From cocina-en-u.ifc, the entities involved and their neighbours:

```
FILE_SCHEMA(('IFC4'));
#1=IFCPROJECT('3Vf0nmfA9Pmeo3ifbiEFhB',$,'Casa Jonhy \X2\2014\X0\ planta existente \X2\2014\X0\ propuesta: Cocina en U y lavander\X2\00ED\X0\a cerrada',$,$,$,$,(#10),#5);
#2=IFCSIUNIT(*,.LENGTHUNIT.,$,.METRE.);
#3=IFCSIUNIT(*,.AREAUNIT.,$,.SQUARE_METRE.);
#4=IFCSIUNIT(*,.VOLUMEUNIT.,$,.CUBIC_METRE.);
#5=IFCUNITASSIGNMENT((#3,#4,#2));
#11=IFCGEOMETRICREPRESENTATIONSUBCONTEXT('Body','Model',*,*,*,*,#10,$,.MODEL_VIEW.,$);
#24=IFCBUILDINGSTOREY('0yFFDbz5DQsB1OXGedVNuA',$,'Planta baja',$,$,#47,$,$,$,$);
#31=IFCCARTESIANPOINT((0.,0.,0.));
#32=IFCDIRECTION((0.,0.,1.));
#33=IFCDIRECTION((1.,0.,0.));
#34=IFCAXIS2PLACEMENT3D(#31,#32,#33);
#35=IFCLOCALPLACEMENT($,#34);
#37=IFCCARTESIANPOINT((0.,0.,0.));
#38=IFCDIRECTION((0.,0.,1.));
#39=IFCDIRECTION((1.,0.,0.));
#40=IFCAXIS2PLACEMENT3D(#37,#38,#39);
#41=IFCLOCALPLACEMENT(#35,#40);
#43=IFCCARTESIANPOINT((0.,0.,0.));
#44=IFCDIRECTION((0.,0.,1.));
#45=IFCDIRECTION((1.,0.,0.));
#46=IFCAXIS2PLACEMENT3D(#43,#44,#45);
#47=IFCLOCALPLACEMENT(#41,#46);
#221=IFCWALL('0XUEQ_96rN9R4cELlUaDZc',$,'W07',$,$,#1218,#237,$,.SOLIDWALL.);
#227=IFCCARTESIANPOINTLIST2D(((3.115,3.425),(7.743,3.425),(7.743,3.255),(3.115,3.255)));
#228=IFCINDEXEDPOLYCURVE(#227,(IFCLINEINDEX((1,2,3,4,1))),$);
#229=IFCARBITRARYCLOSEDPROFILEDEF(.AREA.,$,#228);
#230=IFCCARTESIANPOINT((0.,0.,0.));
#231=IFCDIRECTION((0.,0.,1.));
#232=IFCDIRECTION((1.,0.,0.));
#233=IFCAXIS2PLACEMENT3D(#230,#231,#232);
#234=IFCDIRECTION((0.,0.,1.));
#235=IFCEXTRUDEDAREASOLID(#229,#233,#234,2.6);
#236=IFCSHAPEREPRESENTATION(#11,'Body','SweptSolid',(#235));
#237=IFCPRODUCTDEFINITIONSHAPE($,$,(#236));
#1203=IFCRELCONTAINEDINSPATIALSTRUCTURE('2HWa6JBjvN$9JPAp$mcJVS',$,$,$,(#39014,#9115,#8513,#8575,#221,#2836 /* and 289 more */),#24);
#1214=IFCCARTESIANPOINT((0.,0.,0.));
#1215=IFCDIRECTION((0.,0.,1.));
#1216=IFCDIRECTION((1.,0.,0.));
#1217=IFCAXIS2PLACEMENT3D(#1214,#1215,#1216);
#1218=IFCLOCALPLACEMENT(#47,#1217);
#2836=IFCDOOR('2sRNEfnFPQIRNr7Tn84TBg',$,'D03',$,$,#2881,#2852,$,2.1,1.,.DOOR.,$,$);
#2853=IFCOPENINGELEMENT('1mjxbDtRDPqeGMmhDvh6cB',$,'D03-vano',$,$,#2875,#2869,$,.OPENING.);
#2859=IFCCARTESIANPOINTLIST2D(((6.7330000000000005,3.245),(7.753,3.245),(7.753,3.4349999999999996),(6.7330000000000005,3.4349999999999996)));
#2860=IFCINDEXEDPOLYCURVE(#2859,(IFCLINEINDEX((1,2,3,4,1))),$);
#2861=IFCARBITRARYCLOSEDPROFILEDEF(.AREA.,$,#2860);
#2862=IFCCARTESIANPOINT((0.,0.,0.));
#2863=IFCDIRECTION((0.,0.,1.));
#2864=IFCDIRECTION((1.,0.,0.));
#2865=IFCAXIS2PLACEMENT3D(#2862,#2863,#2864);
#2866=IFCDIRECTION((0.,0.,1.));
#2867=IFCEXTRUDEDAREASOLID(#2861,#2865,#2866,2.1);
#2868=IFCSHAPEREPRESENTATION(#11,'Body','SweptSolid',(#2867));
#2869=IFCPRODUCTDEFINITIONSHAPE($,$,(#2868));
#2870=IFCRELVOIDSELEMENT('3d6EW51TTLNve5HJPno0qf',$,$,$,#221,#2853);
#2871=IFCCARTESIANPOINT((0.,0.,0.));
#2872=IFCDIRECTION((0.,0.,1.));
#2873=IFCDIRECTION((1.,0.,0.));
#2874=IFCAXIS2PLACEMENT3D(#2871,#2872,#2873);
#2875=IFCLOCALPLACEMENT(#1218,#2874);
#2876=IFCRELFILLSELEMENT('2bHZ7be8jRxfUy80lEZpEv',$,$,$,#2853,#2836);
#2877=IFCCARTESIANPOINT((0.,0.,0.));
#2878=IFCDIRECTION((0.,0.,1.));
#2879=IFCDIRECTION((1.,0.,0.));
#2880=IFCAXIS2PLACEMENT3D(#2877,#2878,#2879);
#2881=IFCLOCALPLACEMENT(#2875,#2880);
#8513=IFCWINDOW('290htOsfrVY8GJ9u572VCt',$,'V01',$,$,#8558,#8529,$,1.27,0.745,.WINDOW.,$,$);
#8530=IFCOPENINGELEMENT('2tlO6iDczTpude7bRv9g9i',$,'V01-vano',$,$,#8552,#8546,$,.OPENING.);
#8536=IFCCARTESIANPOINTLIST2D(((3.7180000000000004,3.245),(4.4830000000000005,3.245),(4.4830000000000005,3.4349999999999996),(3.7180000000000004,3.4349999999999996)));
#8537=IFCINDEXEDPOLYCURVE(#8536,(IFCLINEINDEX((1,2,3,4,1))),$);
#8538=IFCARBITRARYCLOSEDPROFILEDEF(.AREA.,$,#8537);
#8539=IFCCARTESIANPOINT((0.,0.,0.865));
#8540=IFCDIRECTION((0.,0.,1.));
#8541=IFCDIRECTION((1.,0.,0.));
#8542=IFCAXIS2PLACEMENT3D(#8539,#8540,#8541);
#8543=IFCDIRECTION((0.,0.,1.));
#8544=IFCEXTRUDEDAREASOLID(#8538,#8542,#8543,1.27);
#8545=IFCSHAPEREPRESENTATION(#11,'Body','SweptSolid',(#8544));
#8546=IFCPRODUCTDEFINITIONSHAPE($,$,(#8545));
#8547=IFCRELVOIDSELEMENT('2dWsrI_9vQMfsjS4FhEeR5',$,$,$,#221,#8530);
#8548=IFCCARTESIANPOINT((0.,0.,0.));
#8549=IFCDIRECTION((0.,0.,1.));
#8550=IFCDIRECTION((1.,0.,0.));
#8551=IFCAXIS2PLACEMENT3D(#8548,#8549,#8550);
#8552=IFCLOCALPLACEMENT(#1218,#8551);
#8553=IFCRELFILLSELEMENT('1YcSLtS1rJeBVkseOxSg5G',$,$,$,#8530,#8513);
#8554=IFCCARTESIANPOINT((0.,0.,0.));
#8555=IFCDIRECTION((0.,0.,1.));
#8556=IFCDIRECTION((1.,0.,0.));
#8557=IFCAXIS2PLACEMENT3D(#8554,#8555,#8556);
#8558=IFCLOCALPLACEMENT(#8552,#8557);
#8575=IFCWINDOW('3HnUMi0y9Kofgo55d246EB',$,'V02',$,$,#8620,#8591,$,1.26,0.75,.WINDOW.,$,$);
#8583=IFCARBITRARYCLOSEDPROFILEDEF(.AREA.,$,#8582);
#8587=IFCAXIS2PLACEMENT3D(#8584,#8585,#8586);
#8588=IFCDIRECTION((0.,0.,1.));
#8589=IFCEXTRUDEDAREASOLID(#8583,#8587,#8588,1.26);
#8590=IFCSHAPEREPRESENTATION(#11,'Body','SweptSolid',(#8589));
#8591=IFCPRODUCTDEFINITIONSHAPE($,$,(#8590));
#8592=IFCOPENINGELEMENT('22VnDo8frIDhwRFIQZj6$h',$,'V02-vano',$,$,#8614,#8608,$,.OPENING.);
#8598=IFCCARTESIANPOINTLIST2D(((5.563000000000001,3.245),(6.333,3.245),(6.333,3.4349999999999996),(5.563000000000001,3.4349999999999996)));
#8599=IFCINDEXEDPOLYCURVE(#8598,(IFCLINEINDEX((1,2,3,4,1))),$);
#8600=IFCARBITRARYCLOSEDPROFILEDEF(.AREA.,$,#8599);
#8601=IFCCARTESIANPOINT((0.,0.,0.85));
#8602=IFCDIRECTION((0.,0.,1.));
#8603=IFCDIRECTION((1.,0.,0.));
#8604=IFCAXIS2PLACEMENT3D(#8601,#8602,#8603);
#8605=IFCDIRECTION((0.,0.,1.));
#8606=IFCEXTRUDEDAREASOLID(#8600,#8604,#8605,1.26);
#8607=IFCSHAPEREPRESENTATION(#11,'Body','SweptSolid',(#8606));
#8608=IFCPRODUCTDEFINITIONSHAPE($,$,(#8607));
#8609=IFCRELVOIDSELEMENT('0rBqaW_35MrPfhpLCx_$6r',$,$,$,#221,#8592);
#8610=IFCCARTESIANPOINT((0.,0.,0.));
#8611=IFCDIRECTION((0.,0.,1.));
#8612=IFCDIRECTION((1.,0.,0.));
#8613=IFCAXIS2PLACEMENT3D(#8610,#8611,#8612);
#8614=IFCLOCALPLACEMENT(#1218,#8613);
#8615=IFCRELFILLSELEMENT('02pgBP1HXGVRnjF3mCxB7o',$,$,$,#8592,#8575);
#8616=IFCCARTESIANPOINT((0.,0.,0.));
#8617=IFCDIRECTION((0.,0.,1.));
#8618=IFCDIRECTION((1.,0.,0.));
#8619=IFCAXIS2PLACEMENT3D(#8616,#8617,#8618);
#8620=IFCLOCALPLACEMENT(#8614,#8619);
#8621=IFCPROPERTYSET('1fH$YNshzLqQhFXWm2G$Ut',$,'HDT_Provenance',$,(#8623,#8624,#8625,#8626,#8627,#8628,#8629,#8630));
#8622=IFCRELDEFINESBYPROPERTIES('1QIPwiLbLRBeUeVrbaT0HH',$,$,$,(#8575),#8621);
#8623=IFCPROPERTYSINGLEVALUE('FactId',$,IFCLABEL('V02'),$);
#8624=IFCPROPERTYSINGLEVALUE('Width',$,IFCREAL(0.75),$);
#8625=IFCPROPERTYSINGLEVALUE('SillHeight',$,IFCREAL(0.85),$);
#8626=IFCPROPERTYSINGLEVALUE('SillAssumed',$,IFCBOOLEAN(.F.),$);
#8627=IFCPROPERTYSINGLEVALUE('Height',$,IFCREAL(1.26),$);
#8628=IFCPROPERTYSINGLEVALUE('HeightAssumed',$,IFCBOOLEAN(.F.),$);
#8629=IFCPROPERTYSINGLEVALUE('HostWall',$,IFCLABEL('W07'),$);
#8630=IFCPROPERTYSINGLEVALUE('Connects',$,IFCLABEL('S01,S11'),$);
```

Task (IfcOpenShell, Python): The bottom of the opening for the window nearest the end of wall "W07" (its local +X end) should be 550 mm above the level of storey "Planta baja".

```python
import numpy as np
import ifcopenshell
import ifcopenshell.api.geometry
import ifcopenshell.api.pset
import ifcopenshell.geom
import ifcopenshell.util.element
import ifcopenshell.util.placement
import ifcopenshell.util.shape
import ifcopenshell.util.unit

model = ifcopenshell.open("cocina-en-u.ifc")
unit_scale = ifcopenshell.util.unit.calculate_unit_scale(model)

window = model.by_guid("3HnUMi0y9Kofgo55d246EB")
opening = window.FillsVoids[0].RelatingOpeningElement
storey = ifcopenshell.util.element.get_container(window, ifc_class="IfcBuildingStorey")
level = ifcopenshell.util.placement.get_local_placement(storey.ObjectPlacement)[2, 3]

# The opening's origin need not be at the sill, so measure its lowest point.
shape = ifcopenshell.geom.create_shape(ifcopenshell.geom.settings(), opening)
bottom = ifcopenshell.util.shape.get_shape_bottom_elevation(shape, shape.geometry) / unit_scale
dz = level + 0.55 / unit_scale - bottom

shift = np.array([0.0, 0.0, dz])
# The window is placed relative to its opening, so it follows when the opening moves.
matrix = ifcopenshell.util.placement.get_local_placement(opening.ObjectPlacement)
matrix[:3, 3] += shift
ifcopenshell.api.geometry.edit_object_placement(
    model, product=opening, matrix=matrix, is_si=False, should_transform_children=True
)

# Keep the stored heights in step.
pset = model.by_id(ifcopenshell.util.element.get_pset(window, "HDT_Provenance", should_inherit=False)["id"])
ifcopenshell.api.pset.edit_pset(model, pset=pset, properties={
    "SillHeight": model.create_entity("IfcReal", ifcopenshell.util.element.get_pset(window, "HDT_Provenance", "SillHeight") + dz),
})

print(f"moved by {dz * unit_scale:+.3f} m")

model.write("cocina-en-u_rev.ifc")
```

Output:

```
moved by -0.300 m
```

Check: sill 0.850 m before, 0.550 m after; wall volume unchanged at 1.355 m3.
